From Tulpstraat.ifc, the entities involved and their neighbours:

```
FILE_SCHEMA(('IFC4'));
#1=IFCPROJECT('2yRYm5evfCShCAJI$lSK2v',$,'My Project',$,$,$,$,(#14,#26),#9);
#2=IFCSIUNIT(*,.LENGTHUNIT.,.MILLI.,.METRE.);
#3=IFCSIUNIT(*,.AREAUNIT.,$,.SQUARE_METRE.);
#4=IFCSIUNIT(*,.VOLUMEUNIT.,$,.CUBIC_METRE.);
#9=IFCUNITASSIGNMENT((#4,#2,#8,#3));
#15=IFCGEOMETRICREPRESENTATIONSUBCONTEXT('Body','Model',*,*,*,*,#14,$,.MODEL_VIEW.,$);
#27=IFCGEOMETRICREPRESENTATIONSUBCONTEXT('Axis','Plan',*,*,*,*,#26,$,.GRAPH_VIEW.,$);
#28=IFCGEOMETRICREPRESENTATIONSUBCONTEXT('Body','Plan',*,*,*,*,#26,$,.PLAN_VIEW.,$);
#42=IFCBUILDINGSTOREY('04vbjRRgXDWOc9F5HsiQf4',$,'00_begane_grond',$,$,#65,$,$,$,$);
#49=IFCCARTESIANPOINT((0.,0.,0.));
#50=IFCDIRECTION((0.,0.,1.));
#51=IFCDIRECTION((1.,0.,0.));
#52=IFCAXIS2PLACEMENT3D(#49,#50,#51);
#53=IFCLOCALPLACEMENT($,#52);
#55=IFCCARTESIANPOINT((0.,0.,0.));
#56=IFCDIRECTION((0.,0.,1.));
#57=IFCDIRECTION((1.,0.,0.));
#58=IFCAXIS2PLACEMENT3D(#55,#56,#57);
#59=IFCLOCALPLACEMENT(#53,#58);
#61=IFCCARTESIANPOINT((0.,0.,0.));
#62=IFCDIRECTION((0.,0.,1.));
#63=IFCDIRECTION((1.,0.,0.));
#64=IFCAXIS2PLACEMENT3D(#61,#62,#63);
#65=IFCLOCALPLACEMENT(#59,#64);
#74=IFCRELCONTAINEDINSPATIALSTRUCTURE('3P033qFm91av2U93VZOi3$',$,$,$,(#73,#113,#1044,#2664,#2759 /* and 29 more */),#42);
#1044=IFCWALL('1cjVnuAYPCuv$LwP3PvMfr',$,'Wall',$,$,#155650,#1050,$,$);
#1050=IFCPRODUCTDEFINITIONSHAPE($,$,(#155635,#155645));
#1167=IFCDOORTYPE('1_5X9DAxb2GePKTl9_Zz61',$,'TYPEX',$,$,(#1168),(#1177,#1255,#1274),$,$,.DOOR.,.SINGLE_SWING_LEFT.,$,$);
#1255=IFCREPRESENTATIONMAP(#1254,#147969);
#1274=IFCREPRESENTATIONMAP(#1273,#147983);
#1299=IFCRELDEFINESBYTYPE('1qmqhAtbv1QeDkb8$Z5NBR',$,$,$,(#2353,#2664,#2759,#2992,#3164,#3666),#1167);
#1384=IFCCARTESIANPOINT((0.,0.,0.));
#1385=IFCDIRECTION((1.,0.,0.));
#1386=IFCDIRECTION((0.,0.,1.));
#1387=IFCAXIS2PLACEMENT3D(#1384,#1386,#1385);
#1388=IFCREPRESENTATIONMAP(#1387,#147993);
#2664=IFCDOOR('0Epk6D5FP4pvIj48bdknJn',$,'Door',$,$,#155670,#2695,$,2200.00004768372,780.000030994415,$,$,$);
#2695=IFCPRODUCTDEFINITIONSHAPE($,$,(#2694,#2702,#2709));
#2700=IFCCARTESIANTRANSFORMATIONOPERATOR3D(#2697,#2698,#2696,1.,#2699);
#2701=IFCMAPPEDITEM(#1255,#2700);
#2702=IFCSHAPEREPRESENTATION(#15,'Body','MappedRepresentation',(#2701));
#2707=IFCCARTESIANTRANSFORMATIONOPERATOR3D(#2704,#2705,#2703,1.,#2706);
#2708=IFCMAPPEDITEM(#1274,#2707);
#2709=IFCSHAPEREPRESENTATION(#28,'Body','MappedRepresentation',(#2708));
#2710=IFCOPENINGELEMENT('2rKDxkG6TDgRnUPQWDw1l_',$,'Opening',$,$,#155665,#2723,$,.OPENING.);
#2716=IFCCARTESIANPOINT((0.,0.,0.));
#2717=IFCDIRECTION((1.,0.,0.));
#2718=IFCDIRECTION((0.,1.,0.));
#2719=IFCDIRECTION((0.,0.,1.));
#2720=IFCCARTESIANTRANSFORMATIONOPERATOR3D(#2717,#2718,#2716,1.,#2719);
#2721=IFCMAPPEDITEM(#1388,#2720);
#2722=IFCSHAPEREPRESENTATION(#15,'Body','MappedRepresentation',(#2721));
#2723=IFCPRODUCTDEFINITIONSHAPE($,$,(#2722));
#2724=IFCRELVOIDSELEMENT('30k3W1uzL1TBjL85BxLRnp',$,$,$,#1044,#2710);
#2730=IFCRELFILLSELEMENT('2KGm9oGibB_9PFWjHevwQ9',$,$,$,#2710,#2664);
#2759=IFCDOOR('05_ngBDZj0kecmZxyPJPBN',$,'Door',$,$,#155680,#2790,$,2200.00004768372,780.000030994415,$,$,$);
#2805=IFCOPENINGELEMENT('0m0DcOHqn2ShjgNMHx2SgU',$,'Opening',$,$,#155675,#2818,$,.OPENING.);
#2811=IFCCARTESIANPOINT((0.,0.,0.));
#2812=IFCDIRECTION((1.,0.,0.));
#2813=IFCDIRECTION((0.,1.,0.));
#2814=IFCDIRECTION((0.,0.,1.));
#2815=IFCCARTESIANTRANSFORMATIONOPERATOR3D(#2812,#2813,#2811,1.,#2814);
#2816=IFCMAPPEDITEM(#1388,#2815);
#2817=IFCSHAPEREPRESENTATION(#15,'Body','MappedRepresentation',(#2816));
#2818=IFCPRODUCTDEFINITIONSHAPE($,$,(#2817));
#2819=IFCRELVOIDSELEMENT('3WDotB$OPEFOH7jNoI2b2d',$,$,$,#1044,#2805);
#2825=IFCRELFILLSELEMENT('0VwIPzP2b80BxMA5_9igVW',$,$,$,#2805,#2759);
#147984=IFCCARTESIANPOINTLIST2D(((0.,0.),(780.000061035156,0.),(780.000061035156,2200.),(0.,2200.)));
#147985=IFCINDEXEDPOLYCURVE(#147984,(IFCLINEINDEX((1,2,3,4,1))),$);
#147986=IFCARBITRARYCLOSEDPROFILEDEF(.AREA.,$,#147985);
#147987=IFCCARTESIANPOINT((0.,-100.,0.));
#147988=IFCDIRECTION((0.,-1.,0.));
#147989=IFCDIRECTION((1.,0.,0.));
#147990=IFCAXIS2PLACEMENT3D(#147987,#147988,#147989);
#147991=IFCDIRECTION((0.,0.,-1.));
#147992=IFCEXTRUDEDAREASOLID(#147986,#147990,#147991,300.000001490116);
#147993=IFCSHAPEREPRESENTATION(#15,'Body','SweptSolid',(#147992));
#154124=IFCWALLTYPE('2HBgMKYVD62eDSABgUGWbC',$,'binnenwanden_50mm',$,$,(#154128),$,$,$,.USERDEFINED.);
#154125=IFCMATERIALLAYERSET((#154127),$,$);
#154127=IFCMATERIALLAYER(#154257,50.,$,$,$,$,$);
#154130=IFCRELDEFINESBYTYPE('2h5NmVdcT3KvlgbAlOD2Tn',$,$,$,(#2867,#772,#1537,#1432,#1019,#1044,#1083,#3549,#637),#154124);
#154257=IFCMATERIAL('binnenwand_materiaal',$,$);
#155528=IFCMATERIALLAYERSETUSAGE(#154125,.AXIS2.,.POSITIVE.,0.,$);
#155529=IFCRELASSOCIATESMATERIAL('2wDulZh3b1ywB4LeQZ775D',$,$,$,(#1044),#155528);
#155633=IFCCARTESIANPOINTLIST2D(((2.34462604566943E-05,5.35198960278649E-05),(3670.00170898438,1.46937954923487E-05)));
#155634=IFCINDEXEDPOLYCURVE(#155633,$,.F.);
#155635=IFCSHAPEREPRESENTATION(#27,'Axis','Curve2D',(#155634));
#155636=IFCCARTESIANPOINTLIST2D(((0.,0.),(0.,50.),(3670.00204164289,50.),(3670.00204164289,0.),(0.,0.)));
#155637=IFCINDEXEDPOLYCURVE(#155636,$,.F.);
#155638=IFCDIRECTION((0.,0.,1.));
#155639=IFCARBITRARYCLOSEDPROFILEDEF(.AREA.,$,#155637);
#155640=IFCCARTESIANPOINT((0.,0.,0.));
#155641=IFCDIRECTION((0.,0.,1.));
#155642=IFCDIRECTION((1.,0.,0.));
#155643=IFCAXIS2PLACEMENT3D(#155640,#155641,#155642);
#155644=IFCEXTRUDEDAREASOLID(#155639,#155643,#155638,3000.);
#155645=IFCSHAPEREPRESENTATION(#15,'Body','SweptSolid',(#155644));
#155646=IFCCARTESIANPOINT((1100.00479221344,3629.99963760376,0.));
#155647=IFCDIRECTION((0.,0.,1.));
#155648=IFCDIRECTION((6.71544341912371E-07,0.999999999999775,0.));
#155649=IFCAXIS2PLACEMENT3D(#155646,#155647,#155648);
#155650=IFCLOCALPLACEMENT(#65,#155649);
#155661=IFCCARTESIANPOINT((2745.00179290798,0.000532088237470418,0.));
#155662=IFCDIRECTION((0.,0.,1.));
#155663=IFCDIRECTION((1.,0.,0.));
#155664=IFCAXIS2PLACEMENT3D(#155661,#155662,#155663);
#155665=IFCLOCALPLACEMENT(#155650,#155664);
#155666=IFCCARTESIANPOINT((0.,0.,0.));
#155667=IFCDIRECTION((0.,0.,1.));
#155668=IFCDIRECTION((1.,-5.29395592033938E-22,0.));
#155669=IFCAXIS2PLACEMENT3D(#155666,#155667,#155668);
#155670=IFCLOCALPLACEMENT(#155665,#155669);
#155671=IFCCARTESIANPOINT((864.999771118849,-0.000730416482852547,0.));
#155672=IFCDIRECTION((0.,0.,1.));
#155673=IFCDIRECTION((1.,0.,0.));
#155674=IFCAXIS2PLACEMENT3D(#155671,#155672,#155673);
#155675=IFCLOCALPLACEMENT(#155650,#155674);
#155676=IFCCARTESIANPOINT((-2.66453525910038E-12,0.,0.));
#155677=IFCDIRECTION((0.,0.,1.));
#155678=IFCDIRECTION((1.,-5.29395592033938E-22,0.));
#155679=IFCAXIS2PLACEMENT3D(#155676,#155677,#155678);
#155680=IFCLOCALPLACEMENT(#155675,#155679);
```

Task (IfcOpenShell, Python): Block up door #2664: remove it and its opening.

```python
import ifcopenshell
import ifcopenshell.api.feature
import ifcopenshell.api.root
import ifcopenshell.geom
import ifcopenshell.util.shape

model = ifcopenshell.open("Tulpstraat.ifc")
settings = ifcopenshell.geom.settings()


def volume(element):
    """Net volume in cubic metres, openings subtracted."""
    shape = ifcopenshell.geom.create_shape(settings, element)
    return ifcopenshell.util.shape.get_volume(shape.geometry)


door = model.by_id(2664)
opening = door.FillsVoids[0].RelatingOpeningElement
wall = opening.VoidsElements[0].RelatingBuildingElement
before = volume(wall)

ifcopenshell.api.root.remove_product(model, product=door)
ifcopenshell.api.feature.remove_feature(model, feature=opening)

after = volume(wall)

print(f"wall volume {before:.3f} -> {after:.3f} m3")

model.write("Tulpstraat-out.ifc")
```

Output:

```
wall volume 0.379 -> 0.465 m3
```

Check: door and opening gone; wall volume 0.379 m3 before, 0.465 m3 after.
